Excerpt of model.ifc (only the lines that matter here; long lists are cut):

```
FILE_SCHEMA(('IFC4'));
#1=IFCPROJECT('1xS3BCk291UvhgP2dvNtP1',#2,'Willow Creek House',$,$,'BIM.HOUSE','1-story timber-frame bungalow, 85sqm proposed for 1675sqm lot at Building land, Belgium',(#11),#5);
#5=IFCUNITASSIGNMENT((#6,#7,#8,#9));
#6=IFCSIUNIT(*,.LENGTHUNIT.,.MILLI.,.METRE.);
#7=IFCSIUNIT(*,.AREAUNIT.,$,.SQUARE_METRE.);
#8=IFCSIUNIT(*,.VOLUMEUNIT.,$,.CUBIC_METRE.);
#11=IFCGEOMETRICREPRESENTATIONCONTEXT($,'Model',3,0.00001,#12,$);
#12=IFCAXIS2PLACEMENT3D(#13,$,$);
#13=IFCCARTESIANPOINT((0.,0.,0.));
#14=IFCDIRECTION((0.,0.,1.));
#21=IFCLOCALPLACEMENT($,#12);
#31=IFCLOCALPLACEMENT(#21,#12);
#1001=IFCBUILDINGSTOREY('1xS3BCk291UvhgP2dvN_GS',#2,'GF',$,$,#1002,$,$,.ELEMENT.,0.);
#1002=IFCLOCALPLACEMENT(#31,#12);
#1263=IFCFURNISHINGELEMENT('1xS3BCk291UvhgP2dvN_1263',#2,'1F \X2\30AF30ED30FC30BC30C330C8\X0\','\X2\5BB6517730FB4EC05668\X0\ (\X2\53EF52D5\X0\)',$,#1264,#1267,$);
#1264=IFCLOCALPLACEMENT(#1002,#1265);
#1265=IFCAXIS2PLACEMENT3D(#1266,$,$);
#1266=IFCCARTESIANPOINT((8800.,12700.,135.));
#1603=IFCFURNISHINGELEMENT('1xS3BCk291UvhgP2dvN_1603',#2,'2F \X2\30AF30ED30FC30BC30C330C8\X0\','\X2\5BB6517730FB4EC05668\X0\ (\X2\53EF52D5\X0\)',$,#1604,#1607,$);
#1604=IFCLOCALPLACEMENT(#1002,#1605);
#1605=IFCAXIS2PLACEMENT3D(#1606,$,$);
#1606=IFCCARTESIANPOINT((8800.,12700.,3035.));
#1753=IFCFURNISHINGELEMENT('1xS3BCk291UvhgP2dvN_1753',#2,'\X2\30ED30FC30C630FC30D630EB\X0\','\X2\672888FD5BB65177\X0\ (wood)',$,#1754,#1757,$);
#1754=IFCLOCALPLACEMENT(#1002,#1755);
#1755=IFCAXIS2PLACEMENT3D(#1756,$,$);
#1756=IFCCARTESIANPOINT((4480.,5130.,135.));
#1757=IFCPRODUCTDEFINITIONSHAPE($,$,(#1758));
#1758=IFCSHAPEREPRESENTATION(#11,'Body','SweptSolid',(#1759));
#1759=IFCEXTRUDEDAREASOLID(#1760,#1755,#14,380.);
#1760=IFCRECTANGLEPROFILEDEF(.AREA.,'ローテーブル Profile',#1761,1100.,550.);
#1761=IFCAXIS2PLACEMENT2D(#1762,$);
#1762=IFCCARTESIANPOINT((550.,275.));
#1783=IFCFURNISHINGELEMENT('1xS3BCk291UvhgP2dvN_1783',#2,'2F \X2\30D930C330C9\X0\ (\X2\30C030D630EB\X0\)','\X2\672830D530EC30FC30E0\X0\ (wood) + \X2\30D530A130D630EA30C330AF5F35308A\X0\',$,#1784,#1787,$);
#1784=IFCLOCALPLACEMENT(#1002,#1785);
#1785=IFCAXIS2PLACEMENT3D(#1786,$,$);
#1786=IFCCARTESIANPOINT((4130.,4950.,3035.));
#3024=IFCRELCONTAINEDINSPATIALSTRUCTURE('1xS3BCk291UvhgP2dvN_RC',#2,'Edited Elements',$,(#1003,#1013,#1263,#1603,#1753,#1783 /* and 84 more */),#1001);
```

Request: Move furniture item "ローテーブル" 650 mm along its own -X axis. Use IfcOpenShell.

```python
import ifcopenshell
import ifcopenshell.api.geometry
import ifcopenshell.util.placement
import ifcopenshell.util.unit

model = ifcopenshell.open("model.ifc")
unit_scale = ifcopenshell.util.unit.calculate_unit_scale(model)

item = model.by_guid("1xS3BCk291UvhgP2dvN_1753")
matrix = ifcopenshell.util.placement.get_local_placement(item.ObjectPlacement)
matrix[:3, 3] -= matrix[:3, 0] * 0.65 / unit_scale
ifcopenshell.api.geometry.edit_object_placement(model, product=item, matrix=matrix, is_si=False)

print(ifcopenshell.util.placement.get_local_placement(item.ObjectPlacement).round(3) + 0.0)

model.write("model_rev.ifc")
```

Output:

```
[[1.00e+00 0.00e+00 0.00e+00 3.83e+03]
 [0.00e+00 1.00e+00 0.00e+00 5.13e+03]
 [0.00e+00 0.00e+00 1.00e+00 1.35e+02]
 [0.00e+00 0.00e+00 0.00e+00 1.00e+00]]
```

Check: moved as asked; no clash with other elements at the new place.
